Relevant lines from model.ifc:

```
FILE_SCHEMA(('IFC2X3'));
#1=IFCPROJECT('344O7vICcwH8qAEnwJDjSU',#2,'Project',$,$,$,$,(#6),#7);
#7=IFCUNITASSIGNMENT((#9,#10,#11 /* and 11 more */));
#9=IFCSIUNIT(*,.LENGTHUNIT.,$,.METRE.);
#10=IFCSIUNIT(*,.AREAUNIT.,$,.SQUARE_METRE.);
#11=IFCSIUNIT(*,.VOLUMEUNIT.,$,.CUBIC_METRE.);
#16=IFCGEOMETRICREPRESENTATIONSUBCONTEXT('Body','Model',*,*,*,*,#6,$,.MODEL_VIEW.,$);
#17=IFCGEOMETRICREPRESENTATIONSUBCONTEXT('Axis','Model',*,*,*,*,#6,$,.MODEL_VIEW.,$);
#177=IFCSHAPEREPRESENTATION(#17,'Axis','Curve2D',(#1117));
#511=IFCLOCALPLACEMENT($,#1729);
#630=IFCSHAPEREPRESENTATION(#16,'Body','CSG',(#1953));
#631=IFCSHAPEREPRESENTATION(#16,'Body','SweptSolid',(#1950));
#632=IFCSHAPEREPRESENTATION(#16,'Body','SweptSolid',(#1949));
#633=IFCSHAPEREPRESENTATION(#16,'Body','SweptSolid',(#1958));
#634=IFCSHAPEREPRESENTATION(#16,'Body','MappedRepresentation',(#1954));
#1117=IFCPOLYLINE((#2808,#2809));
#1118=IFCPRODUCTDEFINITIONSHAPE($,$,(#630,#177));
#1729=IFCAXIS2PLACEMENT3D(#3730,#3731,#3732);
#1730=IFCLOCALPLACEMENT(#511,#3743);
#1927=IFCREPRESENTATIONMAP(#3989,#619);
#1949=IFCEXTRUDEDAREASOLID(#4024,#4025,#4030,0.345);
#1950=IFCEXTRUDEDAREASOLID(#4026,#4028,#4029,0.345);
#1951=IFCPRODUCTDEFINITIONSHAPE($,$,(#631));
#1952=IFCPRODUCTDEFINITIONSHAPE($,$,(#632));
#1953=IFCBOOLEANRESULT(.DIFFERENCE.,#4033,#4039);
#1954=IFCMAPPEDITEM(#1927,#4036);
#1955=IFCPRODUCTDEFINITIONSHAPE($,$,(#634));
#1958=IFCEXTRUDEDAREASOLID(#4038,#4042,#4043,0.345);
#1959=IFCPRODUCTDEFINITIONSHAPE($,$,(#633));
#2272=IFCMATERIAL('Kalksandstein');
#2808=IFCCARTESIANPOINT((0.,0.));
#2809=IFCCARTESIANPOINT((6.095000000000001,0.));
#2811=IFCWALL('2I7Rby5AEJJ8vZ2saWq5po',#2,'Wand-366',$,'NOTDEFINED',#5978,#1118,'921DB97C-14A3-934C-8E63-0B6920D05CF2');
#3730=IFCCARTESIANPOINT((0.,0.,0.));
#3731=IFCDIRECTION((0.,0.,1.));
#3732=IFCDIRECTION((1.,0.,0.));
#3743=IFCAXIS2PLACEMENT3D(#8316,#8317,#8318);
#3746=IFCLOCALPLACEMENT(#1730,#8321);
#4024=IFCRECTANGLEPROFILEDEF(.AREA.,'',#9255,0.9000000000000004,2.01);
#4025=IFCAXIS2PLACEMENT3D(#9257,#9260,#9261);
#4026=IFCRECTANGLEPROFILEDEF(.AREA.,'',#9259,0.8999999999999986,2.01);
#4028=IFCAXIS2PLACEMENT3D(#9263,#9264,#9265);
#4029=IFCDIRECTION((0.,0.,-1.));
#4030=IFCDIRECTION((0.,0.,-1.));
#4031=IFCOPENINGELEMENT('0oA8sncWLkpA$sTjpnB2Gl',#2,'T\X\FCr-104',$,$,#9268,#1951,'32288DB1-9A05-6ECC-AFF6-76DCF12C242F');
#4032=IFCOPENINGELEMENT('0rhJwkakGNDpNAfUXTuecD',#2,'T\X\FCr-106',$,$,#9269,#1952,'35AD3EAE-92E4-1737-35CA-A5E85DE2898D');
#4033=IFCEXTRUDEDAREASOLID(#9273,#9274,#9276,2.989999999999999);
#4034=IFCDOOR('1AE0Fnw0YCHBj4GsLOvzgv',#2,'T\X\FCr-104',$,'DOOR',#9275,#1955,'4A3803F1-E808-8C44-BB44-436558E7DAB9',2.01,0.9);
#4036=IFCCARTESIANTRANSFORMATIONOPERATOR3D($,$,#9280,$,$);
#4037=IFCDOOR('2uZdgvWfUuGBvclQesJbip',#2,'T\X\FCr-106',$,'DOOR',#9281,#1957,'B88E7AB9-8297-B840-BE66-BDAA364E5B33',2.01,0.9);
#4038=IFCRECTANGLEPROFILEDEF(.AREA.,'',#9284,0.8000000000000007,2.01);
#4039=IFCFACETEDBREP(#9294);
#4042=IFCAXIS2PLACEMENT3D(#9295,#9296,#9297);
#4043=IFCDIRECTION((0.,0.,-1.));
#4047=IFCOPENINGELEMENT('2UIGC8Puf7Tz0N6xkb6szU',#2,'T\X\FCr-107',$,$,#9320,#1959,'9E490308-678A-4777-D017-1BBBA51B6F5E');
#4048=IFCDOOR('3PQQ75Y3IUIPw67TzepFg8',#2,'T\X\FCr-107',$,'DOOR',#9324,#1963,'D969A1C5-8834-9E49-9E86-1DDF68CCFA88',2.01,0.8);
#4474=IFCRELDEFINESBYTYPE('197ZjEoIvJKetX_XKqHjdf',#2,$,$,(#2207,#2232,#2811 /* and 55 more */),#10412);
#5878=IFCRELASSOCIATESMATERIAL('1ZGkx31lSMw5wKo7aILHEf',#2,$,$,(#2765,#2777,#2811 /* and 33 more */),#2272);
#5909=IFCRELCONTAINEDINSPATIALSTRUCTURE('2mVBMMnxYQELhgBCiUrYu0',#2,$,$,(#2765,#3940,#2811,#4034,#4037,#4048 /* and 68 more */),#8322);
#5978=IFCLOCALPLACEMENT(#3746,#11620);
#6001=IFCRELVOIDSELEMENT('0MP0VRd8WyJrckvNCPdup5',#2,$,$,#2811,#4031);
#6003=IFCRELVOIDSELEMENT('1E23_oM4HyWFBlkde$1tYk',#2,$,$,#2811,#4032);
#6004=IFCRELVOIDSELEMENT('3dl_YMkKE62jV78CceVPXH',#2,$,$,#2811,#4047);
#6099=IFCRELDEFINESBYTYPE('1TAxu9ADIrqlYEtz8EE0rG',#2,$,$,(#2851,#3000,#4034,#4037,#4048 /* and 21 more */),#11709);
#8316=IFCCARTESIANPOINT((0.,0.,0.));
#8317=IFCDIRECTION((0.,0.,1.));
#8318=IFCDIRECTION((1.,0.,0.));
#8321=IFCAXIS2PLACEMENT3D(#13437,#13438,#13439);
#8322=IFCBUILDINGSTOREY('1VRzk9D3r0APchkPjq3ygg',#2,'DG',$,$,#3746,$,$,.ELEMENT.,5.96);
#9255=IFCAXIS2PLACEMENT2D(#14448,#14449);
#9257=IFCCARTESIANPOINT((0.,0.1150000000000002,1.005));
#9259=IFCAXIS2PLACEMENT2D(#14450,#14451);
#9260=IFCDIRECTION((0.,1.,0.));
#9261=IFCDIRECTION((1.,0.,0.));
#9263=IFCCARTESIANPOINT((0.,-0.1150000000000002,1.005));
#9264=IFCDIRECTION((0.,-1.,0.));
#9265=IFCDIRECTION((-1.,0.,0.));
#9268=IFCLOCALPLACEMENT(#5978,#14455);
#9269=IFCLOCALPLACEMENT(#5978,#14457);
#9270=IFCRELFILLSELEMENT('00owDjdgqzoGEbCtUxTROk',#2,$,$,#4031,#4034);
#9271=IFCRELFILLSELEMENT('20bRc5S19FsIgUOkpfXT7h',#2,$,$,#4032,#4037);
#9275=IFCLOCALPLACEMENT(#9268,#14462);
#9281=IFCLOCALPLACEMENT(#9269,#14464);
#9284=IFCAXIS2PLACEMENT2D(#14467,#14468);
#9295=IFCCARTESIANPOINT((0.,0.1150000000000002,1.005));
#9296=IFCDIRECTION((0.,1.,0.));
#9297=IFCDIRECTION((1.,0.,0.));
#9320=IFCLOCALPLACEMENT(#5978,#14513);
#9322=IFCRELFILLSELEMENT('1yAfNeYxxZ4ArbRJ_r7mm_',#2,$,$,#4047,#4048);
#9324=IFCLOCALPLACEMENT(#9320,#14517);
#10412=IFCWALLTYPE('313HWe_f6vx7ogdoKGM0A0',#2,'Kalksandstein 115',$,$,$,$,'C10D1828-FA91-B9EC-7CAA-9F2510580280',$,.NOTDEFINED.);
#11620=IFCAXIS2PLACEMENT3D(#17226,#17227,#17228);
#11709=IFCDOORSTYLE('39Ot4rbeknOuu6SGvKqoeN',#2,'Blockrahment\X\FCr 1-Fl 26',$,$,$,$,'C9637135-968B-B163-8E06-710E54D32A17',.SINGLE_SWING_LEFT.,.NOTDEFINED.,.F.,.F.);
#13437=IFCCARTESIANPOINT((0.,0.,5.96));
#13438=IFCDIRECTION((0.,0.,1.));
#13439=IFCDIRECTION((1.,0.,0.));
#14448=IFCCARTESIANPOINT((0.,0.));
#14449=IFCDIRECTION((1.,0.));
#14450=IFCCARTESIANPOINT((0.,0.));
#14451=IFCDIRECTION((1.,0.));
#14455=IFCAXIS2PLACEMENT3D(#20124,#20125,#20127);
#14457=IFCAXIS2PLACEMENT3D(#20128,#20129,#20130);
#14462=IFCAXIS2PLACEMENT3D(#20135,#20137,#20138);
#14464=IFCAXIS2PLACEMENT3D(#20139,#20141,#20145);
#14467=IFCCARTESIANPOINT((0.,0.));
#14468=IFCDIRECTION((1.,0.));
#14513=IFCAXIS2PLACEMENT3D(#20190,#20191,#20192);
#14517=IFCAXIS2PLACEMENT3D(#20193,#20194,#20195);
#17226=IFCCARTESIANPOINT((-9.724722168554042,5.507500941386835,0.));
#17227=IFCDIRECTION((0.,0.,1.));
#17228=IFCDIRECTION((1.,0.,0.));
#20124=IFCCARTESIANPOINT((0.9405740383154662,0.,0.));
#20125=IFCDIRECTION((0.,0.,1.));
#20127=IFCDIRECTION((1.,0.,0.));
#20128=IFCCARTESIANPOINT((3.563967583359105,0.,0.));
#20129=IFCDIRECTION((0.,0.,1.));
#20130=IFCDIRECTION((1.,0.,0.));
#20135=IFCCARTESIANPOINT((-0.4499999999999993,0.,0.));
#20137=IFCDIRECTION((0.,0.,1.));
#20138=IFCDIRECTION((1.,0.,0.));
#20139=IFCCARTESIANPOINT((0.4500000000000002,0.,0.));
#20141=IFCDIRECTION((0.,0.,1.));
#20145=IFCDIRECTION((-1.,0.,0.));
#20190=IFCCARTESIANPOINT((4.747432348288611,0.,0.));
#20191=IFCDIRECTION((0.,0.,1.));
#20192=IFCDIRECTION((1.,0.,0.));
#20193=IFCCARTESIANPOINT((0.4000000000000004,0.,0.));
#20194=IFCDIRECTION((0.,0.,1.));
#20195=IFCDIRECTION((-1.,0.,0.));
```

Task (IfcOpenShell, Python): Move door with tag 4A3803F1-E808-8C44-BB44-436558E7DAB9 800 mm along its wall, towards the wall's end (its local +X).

```python
import ifcopenshell
import ifcopenshell.api.geometry
import ifcopenshell.util.placement
import ifcopenshell.util.unit

model = ifcopenshell.open("model.ifc")
unit_scale = ifcopenshell.util.unit.calculate_unit_scale(model)

door = model.by_id(4034)
opening = door.FillsVoids[0].RelatingOpeningElement
wall = opening.VoidsElements[0].RelatingBuildingElement

wall_matrix = ifcopenshell.util.placement.get_local_placement(wall.ObjectPlacement)
shift = wall_matrix[:3, 0] * 0.8 / unit_scale
before = ifcopenshell.util.placement.get_local_placement(door.ObjectPlacement)[:3, 3].copy()

# The door is placed relative to its opening, so it follows when the opening moves.
matrix = ifcopenshell.util.placement.get_local_placement(opening.ObjectPlacement)
matrix[:3, 3] += shift
ifcopenshell.api.geometry.edit_object_placement(
    model, product=opening, matrix=matrix, is_si=False, should_transform_children=True
)

after = ifcopenshell.util.placement.get_local_placement(door.ObjectPlacement)[:3, 3]
print("door moved by", (after - before).round(3) + 0.0)

model.write("model-out.ifc")
```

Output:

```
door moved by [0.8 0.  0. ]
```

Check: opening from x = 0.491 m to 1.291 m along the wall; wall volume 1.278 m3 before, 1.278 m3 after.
